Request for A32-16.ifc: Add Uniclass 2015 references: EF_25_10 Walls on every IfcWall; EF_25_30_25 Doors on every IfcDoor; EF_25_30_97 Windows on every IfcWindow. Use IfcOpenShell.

First a look at what the model holds.

```python
import ifcopenshell

model = ifcopenshell.open("A32-16.ifc")
print(model.schema)
print("classifications:", [c.Name for c in model.by_type("IfcClassification")])
for ifc_class in ("IfcDoor", "IfcRoof", "IfcStair", "IfcWall", "IfcWindow"):
    print(ifc_class, len(model.by_type(ifc_class)))
```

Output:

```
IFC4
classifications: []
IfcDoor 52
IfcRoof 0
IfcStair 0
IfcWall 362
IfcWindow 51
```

```python
import ifcopenshell
import ifcopenshell.api.classification

model = ifcopenshell.open("A32-16.ifc")

system = ifcopenshell.api.classification.add_classification(model, classification="Uniclass 2015")

codes = {
    "IfcWall": ("EF_25_10", "Walls"),
    "IfcDoor": ("EF_25_30_25", "Doors"),
    "IfcWindow": ("EF_25_30_97", "Windows"),
}
for ifc_class, (code, name) in codes.items():
    products = model.by_type(ifc_class)
    ifcopenshell.api.classification.add_reference(
        model, products=products, classification=system, identification=code, name=name
    )
    print(code, len(products))

model.write("A32-16_rev.ifc")
```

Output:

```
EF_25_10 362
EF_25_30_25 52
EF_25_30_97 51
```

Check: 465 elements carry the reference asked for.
